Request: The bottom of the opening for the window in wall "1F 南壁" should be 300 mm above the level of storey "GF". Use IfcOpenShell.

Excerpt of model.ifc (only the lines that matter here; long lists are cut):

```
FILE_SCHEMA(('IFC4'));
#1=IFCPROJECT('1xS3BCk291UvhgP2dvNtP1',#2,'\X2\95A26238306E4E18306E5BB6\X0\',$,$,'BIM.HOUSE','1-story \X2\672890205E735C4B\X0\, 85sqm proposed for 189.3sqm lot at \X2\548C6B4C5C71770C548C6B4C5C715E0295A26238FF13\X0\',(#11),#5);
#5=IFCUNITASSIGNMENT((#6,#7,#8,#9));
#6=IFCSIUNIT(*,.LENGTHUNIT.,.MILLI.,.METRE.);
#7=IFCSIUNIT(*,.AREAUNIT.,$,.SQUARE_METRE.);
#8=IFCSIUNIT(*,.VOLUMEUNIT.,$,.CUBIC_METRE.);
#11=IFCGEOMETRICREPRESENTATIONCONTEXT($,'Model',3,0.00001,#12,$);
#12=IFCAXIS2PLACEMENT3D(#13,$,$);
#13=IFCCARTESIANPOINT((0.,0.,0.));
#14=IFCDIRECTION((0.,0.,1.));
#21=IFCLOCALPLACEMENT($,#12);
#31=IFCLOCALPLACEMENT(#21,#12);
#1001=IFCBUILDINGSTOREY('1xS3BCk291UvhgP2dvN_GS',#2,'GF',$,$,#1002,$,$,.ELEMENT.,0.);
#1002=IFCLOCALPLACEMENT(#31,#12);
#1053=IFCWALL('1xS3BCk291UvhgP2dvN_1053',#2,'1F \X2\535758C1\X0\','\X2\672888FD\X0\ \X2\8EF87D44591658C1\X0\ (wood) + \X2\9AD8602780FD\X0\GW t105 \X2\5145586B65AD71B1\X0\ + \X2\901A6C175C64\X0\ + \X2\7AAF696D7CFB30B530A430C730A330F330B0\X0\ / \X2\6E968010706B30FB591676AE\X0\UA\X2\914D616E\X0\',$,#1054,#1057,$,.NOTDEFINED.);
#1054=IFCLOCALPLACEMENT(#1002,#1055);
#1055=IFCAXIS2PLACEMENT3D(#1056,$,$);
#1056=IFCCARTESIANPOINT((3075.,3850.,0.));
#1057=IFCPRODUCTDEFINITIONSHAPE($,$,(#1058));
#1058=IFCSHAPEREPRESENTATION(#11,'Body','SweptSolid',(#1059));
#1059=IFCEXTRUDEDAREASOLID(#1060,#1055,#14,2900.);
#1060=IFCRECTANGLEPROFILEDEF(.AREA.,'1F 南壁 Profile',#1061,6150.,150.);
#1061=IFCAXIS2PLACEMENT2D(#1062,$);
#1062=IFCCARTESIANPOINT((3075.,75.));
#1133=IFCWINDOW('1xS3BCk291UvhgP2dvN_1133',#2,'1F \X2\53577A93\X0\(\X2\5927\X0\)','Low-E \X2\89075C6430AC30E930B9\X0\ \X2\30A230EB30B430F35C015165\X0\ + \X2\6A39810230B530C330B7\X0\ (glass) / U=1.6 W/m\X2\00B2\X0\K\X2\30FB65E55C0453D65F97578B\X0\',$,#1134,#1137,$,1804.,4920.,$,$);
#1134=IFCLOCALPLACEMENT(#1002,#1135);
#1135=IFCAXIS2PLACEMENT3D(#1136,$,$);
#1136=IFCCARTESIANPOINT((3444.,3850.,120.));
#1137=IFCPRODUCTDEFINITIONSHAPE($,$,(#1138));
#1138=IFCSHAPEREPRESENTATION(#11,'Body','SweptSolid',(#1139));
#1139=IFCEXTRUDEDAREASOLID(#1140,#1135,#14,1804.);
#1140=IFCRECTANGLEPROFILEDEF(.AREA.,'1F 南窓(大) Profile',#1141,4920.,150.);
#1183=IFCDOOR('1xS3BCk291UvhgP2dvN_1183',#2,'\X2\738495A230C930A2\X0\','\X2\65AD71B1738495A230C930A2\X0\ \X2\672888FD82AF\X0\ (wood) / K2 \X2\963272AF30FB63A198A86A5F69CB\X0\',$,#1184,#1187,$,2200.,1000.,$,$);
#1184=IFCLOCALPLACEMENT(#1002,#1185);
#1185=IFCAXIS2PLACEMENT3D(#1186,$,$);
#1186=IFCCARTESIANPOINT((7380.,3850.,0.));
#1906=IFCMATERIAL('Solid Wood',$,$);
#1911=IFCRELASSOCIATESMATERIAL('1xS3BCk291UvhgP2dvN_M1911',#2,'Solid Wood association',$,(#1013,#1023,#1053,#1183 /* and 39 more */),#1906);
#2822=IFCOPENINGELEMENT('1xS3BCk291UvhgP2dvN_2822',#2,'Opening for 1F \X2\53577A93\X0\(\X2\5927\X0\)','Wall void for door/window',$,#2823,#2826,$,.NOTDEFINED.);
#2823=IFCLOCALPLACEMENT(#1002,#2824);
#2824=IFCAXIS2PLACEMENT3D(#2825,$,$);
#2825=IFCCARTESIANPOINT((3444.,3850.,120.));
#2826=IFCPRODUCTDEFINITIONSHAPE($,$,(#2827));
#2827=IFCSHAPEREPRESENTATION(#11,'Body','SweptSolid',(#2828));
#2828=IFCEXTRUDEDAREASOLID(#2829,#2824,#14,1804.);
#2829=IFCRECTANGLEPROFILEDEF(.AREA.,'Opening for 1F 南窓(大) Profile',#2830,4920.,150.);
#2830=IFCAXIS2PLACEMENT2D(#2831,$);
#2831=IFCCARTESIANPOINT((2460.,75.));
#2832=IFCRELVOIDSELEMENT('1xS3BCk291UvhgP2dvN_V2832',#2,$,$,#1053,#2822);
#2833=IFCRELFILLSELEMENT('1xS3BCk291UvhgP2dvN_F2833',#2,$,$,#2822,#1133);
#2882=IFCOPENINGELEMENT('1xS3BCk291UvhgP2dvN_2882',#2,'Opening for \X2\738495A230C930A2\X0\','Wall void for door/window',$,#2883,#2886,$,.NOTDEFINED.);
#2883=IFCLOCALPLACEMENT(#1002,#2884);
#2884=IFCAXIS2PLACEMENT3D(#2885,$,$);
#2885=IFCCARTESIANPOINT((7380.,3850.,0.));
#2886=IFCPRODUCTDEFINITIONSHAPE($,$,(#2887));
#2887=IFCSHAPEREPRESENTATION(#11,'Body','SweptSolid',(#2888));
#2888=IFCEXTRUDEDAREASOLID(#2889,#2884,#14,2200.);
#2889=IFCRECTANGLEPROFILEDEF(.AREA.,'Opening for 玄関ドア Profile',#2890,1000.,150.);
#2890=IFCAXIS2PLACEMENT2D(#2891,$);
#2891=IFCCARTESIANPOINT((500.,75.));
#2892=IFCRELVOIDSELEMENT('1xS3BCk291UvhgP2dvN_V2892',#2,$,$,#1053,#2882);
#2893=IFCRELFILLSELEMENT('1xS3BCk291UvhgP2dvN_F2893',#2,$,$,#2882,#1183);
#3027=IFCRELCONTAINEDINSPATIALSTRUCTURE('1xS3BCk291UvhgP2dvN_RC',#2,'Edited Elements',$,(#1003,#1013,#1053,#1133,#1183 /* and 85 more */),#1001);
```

```python
import numpy as np
import ifcopenshell
import ifcopenshell.api.geometry
import ifcopenshell.geom
import ifcopenshell.util.element
import ifcopenshell.util.placement
import ifcopenshell.util.shape
import ifcopenshell.util.unit

model = ifcopenshell.open("model.ifc")
unit_scale = ifcopenshell.util.unit.calculate_unit_scale(model)

window = model.by_guid("1xS3BCk291UvhgP2dvN_1133")
opening = window.FillsVoids[0].RelatingOpeningElement
storey = ifcopenshell.util.element.get_container(window, ifc_class="IfcBuildingStorey")
level = ifcopenshell.util.placement.get_local_placement(storey.ObjectPlacement)[2, 3]

# The opening's origin need not be at the sill, so measure its lowest point.
shape = ifcopenshell.geom.create_shape(ifcopenshell.geom.settings(), opening)
bottom = ifcopenshell.util.shape.get_shape_bottom_elevation(shape, shape.geometry) / unit_scale
dz = level + 0.3 / unit_scale - bottom

shift = np.array([0.0, 0.0, dz])
# The window is not placed relative to its opening, so move both.
for product in (opening, window):
    matrix = ifcopenshell.util.placement.get_local_placement(product.ObjectPlacement)
    matrix[:3, 3] += shift
    ifcopenshell.api.geometry.edit_object_placement(model, product=product, matrix=matrix, is_si=False)

print(f"moved by {dz * unit_scale:+.3f} m")

model.write("model_edited.ifc")
```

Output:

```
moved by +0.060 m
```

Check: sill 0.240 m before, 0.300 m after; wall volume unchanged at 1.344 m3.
